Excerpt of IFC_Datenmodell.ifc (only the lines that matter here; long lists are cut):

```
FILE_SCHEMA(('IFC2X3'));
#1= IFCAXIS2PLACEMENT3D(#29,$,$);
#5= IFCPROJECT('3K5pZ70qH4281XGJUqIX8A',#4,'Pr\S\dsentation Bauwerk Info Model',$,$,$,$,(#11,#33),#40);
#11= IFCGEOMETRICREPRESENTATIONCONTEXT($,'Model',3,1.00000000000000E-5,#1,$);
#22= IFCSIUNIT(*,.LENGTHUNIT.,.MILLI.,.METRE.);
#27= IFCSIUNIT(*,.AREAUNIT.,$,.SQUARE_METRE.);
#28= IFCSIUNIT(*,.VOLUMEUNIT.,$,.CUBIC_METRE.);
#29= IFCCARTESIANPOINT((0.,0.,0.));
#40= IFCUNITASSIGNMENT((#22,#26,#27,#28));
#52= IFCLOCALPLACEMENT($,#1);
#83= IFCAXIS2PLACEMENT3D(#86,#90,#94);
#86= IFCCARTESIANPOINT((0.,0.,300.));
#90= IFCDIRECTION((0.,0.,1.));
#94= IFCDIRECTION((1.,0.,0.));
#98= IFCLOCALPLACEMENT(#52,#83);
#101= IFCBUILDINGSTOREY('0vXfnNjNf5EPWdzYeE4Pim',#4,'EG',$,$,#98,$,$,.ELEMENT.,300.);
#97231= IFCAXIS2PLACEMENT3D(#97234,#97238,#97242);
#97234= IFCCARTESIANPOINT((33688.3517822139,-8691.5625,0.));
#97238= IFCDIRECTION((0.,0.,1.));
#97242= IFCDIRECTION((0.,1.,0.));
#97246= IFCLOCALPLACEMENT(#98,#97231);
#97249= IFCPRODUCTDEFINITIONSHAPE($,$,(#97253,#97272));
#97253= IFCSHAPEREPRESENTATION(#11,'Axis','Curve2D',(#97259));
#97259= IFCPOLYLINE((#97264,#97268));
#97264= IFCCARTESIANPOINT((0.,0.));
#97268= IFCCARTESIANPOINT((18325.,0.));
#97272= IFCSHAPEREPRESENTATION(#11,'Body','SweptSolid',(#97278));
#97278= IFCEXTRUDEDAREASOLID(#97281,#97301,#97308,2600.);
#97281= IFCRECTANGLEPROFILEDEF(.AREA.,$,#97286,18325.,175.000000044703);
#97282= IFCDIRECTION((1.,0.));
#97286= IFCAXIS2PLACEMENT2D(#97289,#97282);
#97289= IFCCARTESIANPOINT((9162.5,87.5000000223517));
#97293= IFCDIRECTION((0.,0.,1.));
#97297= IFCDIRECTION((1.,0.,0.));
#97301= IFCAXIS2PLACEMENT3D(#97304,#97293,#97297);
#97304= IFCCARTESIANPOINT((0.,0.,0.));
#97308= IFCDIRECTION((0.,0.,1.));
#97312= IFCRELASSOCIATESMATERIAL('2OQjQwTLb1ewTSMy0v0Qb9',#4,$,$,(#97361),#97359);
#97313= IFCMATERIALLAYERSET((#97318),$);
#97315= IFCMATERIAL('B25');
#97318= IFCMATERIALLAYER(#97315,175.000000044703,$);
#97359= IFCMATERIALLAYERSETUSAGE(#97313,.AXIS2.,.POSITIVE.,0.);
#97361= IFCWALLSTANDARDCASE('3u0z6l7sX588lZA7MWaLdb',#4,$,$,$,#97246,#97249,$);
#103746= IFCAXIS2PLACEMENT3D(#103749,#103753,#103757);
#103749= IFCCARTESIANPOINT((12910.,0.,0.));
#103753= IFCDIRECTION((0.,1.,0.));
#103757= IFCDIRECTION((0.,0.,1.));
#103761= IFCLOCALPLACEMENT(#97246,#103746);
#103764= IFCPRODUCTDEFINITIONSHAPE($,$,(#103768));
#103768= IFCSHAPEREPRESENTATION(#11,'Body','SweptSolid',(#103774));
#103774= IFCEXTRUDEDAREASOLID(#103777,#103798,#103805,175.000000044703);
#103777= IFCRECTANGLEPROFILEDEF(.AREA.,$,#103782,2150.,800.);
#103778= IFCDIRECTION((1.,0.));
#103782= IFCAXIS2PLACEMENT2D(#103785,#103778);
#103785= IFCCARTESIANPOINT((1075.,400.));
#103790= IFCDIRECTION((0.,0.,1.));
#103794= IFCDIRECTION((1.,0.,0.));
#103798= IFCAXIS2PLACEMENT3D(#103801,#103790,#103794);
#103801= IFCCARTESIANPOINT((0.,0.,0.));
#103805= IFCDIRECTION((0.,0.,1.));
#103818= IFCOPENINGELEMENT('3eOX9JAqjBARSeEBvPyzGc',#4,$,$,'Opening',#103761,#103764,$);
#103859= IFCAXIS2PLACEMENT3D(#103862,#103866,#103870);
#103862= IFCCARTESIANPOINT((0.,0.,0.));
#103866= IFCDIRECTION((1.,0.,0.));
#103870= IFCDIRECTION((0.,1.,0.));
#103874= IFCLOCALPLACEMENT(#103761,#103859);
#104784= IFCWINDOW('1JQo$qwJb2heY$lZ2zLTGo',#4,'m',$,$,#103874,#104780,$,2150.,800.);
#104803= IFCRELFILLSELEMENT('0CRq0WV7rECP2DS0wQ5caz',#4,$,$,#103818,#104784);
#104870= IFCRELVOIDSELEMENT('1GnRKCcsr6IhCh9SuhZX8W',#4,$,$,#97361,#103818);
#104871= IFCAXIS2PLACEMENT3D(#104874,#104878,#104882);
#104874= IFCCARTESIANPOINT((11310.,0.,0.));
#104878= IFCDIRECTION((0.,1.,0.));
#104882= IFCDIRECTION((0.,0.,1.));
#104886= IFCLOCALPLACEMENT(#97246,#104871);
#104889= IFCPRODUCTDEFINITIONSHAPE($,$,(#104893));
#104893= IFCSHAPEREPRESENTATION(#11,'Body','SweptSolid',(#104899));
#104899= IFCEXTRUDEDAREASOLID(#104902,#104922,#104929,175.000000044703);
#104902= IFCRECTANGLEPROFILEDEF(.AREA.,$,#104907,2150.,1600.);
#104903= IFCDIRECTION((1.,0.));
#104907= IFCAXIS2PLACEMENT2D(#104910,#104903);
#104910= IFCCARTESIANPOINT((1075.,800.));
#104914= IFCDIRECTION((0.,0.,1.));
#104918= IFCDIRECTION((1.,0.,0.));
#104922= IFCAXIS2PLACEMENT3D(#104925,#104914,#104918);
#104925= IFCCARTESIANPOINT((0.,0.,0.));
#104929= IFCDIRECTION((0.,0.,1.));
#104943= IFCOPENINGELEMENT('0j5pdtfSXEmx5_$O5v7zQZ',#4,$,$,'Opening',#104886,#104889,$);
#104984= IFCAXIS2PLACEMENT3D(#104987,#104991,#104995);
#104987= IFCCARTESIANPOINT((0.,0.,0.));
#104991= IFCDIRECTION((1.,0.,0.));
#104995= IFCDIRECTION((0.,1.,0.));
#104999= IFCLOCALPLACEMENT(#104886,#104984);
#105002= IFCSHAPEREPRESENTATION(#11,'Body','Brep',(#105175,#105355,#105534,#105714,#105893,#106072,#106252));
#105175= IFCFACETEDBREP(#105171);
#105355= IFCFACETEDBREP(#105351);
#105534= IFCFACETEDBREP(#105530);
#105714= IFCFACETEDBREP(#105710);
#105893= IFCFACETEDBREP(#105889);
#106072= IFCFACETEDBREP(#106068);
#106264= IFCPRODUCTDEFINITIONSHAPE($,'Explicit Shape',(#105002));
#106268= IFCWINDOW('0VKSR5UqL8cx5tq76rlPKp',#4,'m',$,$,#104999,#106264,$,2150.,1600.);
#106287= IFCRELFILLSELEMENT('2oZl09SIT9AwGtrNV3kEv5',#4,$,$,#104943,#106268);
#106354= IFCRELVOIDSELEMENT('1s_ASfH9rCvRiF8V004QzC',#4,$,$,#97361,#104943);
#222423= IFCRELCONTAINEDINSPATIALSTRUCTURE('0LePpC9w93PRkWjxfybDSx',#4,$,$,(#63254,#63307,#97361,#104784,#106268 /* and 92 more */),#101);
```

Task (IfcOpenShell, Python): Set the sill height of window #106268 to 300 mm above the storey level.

```python
import numpy as np
import ifcopenshell
import ifcopenshell.api.geometry
import ifcopenshell.geom
import ifcopenshell.util.element
import ifcopenshell.util.placement
import ifcopenshell.util.shape
import ifcopenshell.util.unit

model = ifcopenshell.open("IFC_Datenmodell.ifc")
unit_scale = ifcopenshell.util.unit.calculate_unit_scale(model)

window = model.by_guid("0VKSR5UqL8cx5tq76rlPKp")
opening = window.FillsVoids[0].RelatingOpeningElement
storey = ifcopenshell.util.element.get_container(window, ifc_class="IfcBuildingStorey")
level = ifcopenshell.util.placement.get_local_placement(storey.ObjectPlacement)[2, 3]

# The opening's origin need not be at the sill, so measure its lowest point.
shape = ifcopenshell.geom.create_shape(ifcopenshell.geom.settings(), opening)
bottom = ifcopenshell.util.shape.get_shape_bottom_elevation(shape, shape.geometry) / unit_scale
dz = level + 300.0 - bottom

shift = np.array([0.0, 0.0, dz])
# The window is placed relative to its opening, so it follows when the opening moves.
matrix = ifcopenshell.util.placement.get_local_placement(opening.ObjectPlacement)
matrix[:3, 3] += shift
ifcopenshell.api.geometry.edit_object_placement(
    model, product=opening, matrix=matrix, is_si=False, should_transform_children=True
)

print(f"moved by {dz * unit_scale:+.3f} m")

model.write("IFC_Datenmodell_v2.ifc")
```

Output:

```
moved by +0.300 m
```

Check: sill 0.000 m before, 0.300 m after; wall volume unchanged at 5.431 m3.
